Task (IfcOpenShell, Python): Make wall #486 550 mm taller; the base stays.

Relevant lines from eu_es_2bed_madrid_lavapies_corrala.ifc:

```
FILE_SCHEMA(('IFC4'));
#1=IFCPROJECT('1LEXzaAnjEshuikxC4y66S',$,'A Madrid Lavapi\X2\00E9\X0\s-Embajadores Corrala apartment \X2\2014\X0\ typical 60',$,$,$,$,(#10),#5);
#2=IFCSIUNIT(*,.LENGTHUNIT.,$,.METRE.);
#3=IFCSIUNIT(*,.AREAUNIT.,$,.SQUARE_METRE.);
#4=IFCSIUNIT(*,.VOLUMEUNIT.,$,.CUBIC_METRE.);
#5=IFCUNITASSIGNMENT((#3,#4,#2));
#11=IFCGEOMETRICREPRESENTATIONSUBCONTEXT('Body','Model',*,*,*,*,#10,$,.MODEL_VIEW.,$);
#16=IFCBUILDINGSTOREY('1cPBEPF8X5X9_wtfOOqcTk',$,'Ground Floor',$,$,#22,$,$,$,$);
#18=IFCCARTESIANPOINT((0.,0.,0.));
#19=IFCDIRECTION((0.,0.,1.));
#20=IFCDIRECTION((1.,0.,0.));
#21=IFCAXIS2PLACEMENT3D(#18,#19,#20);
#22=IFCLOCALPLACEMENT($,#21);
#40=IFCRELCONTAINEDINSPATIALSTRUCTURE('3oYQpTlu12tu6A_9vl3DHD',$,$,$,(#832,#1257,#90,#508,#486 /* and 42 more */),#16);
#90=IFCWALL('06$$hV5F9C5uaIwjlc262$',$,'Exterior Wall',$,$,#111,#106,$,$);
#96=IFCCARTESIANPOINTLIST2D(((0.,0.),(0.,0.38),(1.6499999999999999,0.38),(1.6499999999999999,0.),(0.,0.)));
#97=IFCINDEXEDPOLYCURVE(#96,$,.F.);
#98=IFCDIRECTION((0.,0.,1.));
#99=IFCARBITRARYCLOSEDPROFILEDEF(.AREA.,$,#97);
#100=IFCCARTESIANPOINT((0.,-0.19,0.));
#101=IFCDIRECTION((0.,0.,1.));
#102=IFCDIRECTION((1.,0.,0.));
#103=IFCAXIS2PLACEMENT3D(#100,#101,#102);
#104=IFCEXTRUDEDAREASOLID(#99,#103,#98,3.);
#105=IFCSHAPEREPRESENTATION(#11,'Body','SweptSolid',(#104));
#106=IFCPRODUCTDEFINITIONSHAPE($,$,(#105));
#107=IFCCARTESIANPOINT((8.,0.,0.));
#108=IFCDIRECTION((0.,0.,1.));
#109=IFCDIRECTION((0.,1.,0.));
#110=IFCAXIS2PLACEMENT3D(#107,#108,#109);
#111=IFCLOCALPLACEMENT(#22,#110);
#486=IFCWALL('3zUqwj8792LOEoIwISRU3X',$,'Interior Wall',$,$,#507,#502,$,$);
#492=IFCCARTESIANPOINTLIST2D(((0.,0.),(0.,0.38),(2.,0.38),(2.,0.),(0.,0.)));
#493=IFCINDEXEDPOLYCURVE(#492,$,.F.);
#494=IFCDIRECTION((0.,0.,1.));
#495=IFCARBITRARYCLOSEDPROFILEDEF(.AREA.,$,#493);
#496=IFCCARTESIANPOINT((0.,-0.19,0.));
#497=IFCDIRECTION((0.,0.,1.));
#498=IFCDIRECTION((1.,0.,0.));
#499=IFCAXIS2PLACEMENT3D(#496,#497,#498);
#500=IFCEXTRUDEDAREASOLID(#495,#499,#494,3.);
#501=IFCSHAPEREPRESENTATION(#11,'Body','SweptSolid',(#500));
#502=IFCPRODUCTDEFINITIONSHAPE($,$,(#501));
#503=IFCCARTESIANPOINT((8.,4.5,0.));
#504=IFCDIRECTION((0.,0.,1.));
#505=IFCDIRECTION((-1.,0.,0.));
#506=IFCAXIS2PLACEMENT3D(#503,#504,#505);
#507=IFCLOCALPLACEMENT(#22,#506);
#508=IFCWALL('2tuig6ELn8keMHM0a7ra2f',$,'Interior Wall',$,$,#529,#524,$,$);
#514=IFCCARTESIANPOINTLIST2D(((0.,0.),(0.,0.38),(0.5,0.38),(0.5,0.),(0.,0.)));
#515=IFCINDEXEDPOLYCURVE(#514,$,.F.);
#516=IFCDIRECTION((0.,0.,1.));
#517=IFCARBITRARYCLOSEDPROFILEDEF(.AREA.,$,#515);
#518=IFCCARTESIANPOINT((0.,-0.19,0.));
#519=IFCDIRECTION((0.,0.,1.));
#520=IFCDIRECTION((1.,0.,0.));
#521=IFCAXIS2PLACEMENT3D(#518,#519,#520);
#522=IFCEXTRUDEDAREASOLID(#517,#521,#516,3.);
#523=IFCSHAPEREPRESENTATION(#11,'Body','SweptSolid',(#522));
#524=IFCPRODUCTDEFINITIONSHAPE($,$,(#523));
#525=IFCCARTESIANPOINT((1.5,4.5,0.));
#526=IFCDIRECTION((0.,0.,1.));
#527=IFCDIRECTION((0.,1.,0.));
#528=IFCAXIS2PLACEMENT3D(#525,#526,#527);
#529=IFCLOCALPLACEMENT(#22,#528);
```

```python
import ifcopenshell
import ifcopenshell.geom
import ifcopenshell.util.representation
import ifcopenshell.util.shape
import ifcopenshell.util.unit

model = ifcopenshell.open("eu_es_2bed_madrid_lavapies_corrala.ifc")
unit_scale = ifcopenshell.util.unit.calculate_unit_scale(model)
settings = ifcopenshell.geom.settings()


def volume(element):
    """Net volume in cubic metres, openings subtracted."""
    shape = ifcopenshell.geom.create_shape(settings, element)
    return ifcopenshell.util.shape.get_volume(shape.geometry)


wall = model.by_id(486)
before = volume(wall)

body = ifcopenshell.util.representation.get_representation(wall, "Model", "Body")
solid = body.Items[0]
old_height = solid.Depth
solid.Depth += 0.55 / unit_scale
after = volume(wall)

print(f"height {old_height:g} -> {solid.Depth:g}, volume {before:.3f} -> {after:.3f} m3")

model.write("eu_es_2bed_madrid_lavapies_corrala_v2.ifc")
```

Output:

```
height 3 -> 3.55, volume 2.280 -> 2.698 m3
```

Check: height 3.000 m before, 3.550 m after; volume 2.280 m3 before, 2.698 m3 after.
